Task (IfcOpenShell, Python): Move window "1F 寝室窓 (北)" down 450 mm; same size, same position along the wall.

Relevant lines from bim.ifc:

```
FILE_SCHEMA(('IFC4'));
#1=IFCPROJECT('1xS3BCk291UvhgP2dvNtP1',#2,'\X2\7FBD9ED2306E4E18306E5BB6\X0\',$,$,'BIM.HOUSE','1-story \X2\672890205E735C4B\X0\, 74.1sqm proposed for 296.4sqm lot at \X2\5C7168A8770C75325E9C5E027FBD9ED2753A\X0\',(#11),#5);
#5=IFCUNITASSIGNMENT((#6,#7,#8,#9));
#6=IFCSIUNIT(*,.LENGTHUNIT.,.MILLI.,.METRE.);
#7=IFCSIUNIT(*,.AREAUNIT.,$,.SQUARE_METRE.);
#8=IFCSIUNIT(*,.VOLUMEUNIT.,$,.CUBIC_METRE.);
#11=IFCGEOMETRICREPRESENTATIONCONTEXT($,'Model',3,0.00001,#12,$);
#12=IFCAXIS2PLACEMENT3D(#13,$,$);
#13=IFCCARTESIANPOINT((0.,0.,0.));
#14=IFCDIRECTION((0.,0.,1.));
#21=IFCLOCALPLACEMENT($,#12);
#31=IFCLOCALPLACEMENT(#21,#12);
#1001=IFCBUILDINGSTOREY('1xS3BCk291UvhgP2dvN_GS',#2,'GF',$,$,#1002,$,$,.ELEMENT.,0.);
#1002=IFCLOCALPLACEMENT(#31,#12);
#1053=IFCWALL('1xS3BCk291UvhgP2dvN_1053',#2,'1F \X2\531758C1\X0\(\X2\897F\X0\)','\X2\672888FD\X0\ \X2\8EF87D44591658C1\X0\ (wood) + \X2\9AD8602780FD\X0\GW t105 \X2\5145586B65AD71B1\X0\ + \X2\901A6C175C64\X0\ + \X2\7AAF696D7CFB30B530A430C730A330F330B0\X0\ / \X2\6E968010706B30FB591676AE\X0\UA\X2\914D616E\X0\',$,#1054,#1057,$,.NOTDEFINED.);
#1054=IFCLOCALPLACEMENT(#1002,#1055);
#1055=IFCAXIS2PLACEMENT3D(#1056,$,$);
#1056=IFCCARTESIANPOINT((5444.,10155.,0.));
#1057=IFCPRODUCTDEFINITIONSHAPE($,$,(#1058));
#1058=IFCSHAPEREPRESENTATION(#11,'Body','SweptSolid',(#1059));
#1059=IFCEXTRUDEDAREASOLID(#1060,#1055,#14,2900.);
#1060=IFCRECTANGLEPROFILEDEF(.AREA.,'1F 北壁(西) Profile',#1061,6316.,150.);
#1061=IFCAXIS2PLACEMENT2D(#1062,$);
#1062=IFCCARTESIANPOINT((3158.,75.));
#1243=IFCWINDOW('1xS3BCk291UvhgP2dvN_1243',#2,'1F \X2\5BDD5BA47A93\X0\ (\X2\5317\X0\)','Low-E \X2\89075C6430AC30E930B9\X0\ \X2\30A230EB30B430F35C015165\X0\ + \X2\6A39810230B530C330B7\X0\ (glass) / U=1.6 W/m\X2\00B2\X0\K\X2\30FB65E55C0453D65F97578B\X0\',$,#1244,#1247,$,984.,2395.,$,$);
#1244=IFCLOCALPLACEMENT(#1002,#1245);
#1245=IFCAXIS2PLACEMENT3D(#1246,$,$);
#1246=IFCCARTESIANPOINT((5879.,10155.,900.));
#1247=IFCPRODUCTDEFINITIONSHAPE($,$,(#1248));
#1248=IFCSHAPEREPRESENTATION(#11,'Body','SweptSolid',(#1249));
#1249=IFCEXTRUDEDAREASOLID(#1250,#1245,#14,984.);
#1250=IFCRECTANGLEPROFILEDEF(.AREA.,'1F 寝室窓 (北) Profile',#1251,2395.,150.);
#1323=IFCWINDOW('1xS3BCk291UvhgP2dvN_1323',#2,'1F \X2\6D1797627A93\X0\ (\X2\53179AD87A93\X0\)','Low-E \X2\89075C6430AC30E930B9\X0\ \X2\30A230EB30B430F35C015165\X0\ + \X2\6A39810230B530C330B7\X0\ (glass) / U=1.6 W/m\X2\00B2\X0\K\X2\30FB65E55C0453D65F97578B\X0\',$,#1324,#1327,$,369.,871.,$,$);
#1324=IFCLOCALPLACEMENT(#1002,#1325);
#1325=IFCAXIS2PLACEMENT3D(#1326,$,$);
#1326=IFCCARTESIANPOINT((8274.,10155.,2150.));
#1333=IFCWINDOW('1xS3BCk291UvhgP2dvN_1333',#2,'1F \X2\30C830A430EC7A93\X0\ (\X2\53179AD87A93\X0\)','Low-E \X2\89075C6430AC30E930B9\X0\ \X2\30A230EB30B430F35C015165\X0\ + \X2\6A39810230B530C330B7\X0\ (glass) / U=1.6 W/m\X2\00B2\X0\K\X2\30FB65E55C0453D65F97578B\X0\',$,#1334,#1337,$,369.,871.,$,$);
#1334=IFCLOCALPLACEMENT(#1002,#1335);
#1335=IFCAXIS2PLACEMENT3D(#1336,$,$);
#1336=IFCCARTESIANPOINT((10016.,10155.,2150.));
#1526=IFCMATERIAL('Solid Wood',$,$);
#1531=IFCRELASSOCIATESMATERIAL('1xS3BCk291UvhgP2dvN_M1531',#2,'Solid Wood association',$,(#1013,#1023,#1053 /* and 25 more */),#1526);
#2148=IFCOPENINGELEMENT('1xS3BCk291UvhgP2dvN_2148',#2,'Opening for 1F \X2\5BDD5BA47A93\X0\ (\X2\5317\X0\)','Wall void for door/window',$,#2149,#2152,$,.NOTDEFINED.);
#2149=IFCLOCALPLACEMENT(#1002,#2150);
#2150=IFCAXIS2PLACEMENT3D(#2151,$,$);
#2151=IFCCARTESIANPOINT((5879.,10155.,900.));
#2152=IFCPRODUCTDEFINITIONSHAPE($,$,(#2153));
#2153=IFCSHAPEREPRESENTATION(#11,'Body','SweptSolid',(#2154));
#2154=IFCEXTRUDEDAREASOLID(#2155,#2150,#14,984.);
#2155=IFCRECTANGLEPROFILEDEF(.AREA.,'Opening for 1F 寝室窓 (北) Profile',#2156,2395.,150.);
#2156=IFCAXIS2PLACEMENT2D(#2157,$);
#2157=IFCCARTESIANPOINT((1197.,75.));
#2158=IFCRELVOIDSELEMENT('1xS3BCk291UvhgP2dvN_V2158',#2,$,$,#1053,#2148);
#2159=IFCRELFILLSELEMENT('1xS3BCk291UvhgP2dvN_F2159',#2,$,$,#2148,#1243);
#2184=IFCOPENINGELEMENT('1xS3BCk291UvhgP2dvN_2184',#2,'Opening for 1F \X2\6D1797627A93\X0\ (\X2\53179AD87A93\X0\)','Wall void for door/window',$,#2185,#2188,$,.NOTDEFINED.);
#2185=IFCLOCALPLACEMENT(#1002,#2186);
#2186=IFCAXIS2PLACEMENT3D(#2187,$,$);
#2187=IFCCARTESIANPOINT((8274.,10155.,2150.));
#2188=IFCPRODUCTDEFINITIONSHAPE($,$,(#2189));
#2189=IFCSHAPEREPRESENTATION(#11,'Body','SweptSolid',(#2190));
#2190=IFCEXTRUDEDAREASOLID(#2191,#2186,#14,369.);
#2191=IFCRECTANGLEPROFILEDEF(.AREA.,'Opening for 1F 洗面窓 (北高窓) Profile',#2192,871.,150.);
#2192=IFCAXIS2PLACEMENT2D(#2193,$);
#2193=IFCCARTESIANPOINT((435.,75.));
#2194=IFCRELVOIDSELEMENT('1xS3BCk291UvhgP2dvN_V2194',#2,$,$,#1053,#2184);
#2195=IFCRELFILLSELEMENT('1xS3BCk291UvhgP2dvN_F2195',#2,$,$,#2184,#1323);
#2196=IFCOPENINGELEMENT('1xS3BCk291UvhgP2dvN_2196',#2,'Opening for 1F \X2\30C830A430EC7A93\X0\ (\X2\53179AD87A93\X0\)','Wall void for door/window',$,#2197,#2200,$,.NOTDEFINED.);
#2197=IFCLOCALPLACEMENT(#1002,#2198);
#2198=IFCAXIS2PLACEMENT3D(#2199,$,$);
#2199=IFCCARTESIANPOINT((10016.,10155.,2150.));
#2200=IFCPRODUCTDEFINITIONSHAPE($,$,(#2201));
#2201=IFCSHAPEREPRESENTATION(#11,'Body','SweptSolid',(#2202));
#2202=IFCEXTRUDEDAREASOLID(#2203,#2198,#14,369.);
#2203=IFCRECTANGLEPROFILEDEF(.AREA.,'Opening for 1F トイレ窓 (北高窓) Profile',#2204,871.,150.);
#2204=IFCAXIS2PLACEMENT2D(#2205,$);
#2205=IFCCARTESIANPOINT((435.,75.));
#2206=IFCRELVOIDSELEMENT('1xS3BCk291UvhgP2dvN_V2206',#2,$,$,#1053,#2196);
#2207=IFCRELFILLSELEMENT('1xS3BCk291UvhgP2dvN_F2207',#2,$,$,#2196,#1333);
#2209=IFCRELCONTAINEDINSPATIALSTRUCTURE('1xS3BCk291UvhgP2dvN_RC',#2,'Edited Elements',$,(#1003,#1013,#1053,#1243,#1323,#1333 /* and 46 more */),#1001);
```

```python
import numpy as np
import ifcopenshell
import ifcopenshell.api.geometry
import ifcopenshell.util.placement
import ifcopenshell.util.unit

model = ifcopenshell.open("bim.ifc")
unit_scale = ifcopenshell.util.unit.calculate_unit_scale(model)

window = model.by_guid("1xS3BCk291UvhgP2dvN_1243")
opening = window.FillsVoids[0].RelatingOpeningElement
dz = -450.0

shift = np.array([0.0, 0.0, dz])
# The window is not placed relative to its opening, so move both.
for product in (opening, window):
    matrix = ifcopenshell.util.placement.get_local_placement(product.ObjectPlacement)
    matrix[:3, 3] += shift
    ifcopenshell.api.geometry.edit_object_placement(model, product=product, matrix=matrix, is_si=False)

print(f"moved by {dz * unit_scale:+.3f} m")

model.write("bim-out.ifc")
```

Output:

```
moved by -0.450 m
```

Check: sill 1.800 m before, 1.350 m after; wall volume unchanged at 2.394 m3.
